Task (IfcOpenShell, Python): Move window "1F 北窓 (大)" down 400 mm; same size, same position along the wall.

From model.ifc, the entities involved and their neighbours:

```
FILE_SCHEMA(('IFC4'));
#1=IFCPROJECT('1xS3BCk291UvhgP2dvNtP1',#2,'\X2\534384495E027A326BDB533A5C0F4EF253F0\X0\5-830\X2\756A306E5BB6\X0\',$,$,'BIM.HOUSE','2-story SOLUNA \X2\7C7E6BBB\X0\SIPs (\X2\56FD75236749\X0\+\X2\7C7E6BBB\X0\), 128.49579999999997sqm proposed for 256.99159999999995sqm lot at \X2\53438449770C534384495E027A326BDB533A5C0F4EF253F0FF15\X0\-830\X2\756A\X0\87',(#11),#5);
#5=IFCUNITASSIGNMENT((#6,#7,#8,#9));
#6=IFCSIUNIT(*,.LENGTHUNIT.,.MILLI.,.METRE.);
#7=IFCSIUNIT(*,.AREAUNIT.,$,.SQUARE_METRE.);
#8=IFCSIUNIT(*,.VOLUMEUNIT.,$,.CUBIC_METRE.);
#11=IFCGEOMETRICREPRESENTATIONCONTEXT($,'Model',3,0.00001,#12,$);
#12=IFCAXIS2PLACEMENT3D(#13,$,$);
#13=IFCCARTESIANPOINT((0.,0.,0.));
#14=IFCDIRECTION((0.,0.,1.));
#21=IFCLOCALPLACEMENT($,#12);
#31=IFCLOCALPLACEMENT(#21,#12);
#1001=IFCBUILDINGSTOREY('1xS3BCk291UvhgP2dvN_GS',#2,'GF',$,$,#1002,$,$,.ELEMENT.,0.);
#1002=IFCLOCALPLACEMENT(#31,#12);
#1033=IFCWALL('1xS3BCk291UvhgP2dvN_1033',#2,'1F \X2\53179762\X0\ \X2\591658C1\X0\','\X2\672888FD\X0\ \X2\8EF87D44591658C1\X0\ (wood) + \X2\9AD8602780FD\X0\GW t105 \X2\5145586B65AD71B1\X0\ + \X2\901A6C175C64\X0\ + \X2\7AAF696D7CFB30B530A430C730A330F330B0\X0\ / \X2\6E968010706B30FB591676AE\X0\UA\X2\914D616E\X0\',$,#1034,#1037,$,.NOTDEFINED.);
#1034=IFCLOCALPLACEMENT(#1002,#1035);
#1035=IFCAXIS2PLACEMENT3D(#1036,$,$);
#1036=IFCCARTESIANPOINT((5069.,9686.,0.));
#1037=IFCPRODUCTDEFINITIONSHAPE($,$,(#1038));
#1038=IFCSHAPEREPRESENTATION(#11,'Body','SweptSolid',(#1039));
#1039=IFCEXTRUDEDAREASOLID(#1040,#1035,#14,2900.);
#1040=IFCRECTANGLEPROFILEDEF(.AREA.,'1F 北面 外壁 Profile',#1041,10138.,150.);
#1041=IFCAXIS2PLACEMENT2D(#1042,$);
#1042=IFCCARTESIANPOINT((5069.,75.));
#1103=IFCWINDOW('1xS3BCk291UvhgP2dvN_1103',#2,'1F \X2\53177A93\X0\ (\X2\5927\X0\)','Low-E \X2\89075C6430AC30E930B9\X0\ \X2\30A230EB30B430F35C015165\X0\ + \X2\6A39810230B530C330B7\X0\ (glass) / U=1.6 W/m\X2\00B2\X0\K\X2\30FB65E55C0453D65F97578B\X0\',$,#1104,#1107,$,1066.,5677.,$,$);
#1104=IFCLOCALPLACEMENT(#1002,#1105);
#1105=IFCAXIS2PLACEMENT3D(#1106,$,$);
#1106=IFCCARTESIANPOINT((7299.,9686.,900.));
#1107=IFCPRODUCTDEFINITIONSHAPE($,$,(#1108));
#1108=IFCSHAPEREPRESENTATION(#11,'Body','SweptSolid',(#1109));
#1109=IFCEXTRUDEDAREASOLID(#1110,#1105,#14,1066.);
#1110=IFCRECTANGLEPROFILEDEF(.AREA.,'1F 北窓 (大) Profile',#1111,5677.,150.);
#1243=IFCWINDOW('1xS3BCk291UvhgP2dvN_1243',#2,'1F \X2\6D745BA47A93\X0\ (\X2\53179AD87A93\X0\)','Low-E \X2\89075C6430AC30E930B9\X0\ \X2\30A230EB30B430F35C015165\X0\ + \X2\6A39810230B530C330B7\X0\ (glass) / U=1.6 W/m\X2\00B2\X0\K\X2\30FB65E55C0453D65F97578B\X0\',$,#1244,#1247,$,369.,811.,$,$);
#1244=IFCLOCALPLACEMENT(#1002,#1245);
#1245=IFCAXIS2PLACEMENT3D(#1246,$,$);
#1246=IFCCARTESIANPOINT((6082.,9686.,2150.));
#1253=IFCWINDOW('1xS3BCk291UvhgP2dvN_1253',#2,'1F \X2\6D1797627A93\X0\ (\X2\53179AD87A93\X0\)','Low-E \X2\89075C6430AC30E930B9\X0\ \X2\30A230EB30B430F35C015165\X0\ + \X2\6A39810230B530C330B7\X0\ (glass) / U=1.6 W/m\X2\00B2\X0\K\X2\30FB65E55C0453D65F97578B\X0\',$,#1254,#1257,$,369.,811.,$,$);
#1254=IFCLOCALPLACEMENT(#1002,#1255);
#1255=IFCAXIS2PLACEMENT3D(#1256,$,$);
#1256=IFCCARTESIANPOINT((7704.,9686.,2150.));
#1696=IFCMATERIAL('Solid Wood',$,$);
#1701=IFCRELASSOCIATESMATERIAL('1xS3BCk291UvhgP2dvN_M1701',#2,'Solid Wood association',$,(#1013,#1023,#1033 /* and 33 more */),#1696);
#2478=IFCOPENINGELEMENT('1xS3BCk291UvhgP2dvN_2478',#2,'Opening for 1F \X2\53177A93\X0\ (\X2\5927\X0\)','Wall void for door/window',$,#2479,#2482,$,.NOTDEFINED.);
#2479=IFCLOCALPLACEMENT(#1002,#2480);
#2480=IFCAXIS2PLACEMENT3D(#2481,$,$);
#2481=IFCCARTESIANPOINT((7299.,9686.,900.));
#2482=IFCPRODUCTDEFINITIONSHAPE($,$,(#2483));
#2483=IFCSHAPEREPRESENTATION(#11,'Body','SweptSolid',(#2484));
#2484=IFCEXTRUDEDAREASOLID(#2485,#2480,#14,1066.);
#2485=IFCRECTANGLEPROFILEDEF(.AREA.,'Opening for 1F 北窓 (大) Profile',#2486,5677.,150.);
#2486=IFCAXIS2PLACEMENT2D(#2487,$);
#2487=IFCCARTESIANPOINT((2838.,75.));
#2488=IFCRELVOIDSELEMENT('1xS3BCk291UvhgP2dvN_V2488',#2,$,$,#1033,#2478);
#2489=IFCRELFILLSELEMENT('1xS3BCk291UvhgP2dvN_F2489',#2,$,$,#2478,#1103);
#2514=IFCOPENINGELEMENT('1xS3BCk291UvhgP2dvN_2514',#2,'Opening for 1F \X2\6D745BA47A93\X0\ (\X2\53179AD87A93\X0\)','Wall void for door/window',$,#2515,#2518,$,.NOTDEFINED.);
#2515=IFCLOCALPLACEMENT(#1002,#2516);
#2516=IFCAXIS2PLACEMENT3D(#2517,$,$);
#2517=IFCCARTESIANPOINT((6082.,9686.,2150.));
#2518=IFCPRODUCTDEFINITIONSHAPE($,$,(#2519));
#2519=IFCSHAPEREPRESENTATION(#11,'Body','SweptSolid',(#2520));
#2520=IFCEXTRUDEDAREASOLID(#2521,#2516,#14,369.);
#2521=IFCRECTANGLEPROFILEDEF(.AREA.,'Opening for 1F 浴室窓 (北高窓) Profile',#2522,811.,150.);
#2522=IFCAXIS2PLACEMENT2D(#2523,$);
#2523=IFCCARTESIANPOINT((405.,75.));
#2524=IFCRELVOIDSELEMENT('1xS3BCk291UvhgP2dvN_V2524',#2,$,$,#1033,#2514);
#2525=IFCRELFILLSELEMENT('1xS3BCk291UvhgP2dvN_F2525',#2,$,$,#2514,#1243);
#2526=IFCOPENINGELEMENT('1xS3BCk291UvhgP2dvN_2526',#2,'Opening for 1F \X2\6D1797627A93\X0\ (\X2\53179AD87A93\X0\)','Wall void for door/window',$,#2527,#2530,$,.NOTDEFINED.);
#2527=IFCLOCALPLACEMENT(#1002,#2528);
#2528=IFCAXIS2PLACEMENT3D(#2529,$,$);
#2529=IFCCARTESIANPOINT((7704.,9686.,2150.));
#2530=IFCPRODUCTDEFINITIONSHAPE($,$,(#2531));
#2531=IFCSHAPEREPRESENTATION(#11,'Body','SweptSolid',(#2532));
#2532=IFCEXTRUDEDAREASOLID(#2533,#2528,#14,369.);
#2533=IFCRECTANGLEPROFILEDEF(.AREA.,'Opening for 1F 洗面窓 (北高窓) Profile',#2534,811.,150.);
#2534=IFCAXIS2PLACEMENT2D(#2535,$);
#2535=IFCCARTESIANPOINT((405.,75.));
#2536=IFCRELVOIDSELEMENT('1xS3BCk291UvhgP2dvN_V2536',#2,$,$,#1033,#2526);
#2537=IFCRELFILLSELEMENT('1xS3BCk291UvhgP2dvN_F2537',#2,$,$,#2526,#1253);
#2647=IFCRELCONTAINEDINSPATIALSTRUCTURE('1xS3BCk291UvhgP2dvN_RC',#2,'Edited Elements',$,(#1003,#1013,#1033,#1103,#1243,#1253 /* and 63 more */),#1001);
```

```python
import numpy as np
import ifcopenshell
import ifcopenshell.api.geometry
import ifcopenshell.util.placement
import ifcopenshell.util.unit

model = ifcopenshell.open("model.ifc")
unit_scale = ifcopenshell.util.unit.calculate_unit_scale(model)

window = model.by_guid("1xS3BCk291UvhgP2dvN_1103")
opening = window.FillsVoids[0].RelatingOpeningElement
dz = -400.0

shift = np.array([0.0, 0.0, dz])
# The window is not placed relative to its opening, so move both.
for product in (opening, window):
    matrix = ifcopenshell.util.placement.get_local_placement(product.ObjectPlacement)
    matrix[:3, 3] += shift
    ifcopenshell.api.geometry.edit_object_placement(model, product=product, matrix=matrix, is_si=False)

print(f"moved by {dz * unit_scale:+.3f} m")

model.write("model_v2.ifc")
```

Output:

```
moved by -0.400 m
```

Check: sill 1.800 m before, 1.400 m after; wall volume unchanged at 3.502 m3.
